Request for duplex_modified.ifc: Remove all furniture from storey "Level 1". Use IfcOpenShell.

First a look at what the model holds.

```python
import ifcopenshell
import ifcopenshell.util.element

model = ifcopenshell.open("duplex_modified.ifc")
print(model.schema)
storey = next(s for s in model.by_type("IfcBuildingStorey") if s.Name == "Level 1")
furniture = [e for e in ifcopenshell.util.element.get_decomposition(storey) if e.is_a("IfcFurnishingElement")]
seen = {}
for e in furniture:
    element_type = ifcopenshell.util.element.get_type(e)
    name = element_type.Name if element_type not in (None, e) else None
    seen[name] = seen.get(name, 0) + 1
for name, count in sorted(seen.items(), key=str):
    print(count, "x", name)
```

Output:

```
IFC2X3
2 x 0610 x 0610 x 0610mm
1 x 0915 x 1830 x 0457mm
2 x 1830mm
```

```python
import ifcopenshell
import ifcopenshell.api.root
import ifcopenshell.util.element

model = ifcopenshell.open("duplex_modified.ifc")

storey = next(s for s in model.by_type("IfcBuildingStorey") if s.Name == "Level 1")
furniture = [e for e in ifcopenshell.util.element.get_decomposition(storey) if e.is_a("IfcFurnishingElement")]

for e in furniture:
    ifcopenshell.api.root.remove_product(model, product=e)
print(len(furniture), "removed")

model.write("duplex_modified_v2.ifc")
```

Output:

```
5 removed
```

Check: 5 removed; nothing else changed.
